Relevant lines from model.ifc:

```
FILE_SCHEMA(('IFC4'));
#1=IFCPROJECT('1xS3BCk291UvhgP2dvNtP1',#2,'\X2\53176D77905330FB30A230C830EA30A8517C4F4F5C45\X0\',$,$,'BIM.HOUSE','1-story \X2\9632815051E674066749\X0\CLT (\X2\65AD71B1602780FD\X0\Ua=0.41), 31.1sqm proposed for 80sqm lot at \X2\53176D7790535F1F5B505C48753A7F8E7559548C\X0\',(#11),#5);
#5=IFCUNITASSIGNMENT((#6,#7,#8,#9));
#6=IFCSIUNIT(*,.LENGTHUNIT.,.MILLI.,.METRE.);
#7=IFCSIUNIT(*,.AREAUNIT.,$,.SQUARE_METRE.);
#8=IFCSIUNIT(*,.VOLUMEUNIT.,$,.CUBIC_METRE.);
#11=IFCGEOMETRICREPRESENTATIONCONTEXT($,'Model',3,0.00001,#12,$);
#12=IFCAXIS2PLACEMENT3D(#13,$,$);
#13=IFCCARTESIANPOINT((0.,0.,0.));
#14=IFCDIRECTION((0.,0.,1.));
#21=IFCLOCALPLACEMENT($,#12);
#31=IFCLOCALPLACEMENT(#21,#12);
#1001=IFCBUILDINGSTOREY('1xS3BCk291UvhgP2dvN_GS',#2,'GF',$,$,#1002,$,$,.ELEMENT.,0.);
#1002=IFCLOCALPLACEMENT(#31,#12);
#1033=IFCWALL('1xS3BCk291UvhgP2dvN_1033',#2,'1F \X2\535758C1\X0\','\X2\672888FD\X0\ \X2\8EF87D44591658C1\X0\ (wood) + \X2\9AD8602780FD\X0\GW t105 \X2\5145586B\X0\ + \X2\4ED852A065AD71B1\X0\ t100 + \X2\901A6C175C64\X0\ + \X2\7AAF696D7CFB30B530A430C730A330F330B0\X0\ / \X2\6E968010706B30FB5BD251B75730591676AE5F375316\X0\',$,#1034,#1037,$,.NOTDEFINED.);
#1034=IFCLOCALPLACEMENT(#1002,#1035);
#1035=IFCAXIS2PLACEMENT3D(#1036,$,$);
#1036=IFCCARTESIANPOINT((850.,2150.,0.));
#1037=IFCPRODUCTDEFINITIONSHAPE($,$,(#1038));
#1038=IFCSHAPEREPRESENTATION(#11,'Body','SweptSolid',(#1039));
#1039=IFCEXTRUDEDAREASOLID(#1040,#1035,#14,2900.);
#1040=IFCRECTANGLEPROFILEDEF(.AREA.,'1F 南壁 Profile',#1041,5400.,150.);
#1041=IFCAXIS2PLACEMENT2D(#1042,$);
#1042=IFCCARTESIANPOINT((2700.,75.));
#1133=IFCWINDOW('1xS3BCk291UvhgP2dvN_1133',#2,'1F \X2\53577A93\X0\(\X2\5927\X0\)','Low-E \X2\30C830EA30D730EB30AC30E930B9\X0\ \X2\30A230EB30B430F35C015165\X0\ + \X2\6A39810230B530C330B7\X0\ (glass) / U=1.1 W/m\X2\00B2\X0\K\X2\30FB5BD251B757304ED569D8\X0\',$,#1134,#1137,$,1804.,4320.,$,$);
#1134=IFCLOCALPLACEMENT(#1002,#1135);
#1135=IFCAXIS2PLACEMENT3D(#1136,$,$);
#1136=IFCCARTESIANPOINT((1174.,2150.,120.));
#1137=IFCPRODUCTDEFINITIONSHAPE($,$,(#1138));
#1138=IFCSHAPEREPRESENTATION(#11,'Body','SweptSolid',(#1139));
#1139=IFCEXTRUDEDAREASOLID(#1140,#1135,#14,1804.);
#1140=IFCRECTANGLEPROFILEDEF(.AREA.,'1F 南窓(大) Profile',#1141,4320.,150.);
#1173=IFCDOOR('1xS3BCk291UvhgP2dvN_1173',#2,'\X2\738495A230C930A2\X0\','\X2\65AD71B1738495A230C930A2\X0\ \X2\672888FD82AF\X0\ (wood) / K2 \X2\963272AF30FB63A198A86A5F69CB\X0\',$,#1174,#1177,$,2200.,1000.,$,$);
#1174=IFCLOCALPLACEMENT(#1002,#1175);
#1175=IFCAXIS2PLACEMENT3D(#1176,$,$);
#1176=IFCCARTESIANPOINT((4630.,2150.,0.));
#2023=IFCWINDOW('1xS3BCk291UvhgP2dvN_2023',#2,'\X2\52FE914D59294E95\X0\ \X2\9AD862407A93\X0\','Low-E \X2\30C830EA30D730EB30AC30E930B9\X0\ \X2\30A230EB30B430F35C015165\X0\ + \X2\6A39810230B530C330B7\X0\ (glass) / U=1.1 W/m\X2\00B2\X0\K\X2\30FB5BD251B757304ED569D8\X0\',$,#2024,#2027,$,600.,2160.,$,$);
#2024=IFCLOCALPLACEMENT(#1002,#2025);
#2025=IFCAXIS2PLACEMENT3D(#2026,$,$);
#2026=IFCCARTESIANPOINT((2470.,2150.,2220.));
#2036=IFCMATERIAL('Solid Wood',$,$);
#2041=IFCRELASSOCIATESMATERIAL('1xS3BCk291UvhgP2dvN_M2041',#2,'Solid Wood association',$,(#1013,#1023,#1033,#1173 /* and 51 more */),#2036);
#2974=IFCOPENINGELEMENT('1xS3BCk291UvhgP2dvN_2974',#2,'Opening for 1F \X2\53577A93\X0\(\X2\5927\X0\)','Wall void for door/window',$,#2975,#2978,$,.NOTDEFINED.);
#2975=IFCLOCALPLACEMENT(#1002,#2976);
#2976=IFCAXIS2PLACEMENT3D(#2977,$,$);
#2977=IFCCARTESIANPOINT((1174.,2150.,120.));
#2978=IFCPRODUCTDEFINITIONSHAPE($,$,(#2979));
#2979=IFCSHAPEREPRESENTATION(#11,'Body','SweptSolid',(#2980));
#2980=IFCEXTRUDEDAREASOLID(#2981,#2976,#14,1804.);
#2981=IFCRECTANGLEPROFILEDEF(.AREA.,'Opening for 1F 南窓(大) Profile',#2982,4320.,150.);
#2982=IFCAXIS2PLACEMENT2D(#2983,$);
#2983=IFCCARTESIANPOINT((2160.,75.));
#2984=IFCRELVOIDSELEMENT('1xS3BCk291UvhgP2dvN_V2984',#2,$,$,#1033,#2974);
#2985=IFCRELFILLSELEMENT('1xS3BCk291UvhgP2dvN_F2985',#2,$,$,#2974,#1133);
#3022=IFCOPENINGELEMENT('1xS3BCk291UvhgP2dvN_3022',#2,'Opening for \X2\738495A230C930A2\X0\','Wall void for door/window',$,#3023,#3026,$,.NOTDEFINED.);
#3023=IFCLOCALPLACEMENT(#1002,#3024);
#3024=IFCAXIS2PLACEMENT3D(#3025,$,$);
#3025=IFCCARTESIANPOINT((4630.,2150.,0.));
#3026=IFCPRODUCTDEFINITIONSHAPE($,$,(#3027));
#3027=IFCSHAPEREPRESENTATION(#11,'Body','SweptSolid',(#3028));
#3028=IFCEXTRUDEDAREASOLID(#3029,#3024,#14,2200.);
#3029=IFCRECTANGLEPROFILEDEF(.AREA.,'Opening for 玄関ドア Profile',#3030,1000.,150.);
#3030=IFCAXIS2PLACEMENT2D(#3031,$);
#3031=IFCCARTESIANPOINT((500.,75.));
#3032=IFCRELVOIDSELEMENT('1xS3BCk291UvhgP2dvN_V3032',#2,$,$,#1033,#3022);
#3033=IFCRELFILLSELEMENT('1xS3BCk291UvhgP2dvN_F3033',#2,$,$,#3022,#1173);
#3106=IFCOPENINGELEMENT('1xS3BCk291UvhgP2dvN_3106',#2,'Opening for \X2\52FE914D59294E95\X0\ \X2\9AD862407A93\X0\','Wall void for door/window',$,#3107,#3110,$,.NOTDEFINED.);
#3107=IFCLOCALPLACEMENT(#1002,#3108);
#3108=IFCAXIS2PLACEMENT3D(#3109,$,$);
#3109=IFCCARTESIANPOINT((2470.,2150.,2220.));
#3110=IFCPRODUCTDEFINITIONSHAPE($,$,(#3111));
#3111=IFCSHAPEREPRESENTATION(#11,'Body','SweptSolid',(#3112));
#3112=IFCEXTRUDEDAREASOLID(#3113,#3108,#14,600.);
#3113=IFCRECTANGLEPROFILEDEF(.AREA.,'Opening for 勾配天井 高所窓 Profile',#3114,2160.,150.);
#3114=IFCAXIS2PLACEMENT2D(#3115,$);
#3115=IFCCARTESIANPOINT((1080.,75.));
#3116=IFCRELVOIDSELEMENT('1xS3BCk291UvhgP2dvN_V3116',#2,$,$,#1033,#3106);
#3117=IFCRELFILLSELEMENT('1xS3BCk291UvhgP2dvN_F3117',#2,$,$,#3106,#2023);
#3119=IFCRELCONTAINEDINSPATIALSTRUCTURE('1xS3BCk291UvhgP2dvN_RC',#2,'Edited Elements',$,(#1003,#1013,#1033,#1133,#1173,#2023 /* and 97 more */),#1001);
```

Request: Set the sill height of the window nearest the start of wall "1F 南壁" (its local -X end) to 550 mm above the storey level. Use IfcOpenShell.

```python
import numpy as np
import ifcopenshell
import ifcopenshell.api.geometry
import ifcopenshell.geom
import ifcopenshell.util.element
import ifcopenshell.util.placement
import ifcopenshell.util.shape
import ifcopenshell.util.unit

model = ifcopenshell.open("model.ifc")
unit_scale = ifcopenshell.util.unit.calculate_unit_scale(model)

window = model.by_guid("1xS3BCk291UvhgP2dvN_1133")
opening = window.FillsVoids[0].RelatingOpeningElement
storey = ifcopenshell.util.element.get_container(window, ifc_class="IfcBuildingStorey")
level = ifcopenshell.util.placement.get_local_placement(storey.ObjectPlacement)[2, 3]

# The opening's origin need not be at the sill, so measure its lowest point.
shape = ifcopenshell.geom.create_shape(ifcopenshell.geom.settings(), opening)
bottom = ifcopenshell.util.shape.get_shape_bottom_elevation(shape, shape.geometry) / unit_scale
dz = level + 0.55 / unit_scale - bottom

shift = np.array([0.0, 0.0, dz])
# The window is not placed relative to its opening, so move both.
for product in (opening, window):
    matrix = ifcopenshell.util.placement.get_local_placement(product.ObjectPlacement)
    matrix[:3, 3] += shift
    ifcopenshell.api.geometry.edit_object_placement(model, product=product, matrix=matrix, is_si=False)

print(f"moved by {dz * unit_scale:+.3f} m")

model.write("model-out.ifc")
```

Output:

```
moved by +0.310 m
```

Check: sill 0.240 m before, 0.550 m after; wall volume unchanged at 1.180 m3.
